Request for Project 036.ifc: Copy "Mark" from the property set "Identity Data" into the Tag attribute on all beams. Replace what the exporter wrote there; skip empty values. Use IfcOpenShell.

First a look at what the model holds.

```python
import ifcopenshell
import ifcopenshell.util.element

model = ifcopenshell.open("Project 036.ifc")
print(model.schema)
beams = model.by_type("IfcBeam")
print(len(beams), "beams")
for e in beams[:8]:
    source = ifcopenshell.util.element.get_pset(e, "Identity Data", "Mark")
    target = e.Tag
    print(e.id(), repr(source), repr(target), sep=" | ")
```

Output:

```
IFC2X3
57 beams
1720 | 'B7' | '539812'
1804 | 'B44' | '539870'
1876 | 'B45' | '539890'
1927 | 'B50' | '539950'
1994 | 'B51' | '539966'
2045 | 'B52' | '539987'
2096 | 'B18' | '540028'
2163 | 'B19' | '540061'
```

```python
import ifcopenshell
import ifcopenshell.util.element

model = ifcopenshell.open("Project 036.ifc")

count = 0
for e in model.by_type("IfcBeam"):
    value = ifcopenshell.util.element.get_pset(e, "Identity Data", "Mark")
    current = e.Tag
    if not value or not value.strip() or current == value:
        continue
    e.Tag = value
    count += 1

print(count, "beams updated")

model.write("Project 036_v2.ifc")
```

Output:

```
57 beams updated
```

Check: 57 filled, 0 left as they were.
